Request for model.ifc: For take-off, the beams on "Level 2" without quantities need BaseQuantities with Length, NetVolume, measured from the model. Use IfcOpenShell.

First a look at what the model holds.

```python
import ifcopenshell
import ifcopenshell.util.element
import ifcopenshell.util.unit

model = ifcopenshell.open("model.ifc")
print(model.schema)
for unit_type in ("LENGTHUNIT", "AREAUNIT", "VOLUMEUNIT"):
    print(unit_type, ifcopenshell.util.unit.calculate_unit_scale(model, unit_type))
storey = next(s for s in model.by_type("IfcBuildingStorey") if s.Name == "Level 2")
beams = [e for e in ifcopenshell.util.element.get_decomposition(storey) if e.is_a("IfcBeam")]
for e in sorted(beams, key=lambda e: e.id()):
    print(e.id(), e.is_a(), e.Name, list(ifcopenshell.util.element.get_psets(e, qtos_only=True)), sep=" | ")
```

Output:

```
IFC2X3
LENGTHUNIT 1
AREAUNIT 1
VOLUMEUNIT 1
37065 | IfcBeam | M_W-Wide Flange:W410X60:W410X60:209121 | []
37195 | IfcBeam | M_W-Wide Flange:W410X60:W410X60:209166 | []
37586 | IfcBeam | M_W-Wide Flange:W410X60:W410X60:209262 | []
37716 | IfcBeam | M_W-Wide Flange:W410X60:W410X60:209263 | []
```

```python
import ifcopenshell
import ifcopenshell.api.pset
import ifcopenshell.geom
import ifcopenshell.util.element
import ifcopenshell.util.shape
import ifcopenshell.util.unit

model = ifcopenshell.open("model.ifc")
unit_scale = ifcopenshell.util.unit.calculate_unit_scale(model)
volume_scale = ifcopenshell.util.unit.calculate_unit_scale(model, "VOLUMEUNIT")
settings = ifcopenshell.geom.settings()

storey = next(s for s in model.by_type("IfcBuildingStorey") if s.Name == "Level 2")
beams = [e for e in ifcopenshell.util.element.get_decomposition(storey) if e.is_a("IfcBeam")]

for e in sorted(beams, key=lambda e: e.id()):
    if ifcopenshell.util.element.get_psets(e, qtos_only=True, should_inherit=False):
        continue
    # Geometry comes back in metres, in the element's own axes.
    shape = ifcopenshell.geom.create_shape(settings, e)
    values = {
        "Length": ifcopenshell.util.shape.get_max_xyz(shape.geometry) / unit_scale,
        "NetVolume": ifcopenshell.util.shape.get_volume(shape.geometry) / volume_scale,
    }
    qto = ifcopenshell.api.pset.add_qto(model, product=e, name="BaseQuantities")
    ifcopenshell.api.pset.edit_qto(model, qto=qto, properties=values)
    print(e.id(), {k: round(v, 3) for k, v in values.items()})

model.write("model-out.ifc")
```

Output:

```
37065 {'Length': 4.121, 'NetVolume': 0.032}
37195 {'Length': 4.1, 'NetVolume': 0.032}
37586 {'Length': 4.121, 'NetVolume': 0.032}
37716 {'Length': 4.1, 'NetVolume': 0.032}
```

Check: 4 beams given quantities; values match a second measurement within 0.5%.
